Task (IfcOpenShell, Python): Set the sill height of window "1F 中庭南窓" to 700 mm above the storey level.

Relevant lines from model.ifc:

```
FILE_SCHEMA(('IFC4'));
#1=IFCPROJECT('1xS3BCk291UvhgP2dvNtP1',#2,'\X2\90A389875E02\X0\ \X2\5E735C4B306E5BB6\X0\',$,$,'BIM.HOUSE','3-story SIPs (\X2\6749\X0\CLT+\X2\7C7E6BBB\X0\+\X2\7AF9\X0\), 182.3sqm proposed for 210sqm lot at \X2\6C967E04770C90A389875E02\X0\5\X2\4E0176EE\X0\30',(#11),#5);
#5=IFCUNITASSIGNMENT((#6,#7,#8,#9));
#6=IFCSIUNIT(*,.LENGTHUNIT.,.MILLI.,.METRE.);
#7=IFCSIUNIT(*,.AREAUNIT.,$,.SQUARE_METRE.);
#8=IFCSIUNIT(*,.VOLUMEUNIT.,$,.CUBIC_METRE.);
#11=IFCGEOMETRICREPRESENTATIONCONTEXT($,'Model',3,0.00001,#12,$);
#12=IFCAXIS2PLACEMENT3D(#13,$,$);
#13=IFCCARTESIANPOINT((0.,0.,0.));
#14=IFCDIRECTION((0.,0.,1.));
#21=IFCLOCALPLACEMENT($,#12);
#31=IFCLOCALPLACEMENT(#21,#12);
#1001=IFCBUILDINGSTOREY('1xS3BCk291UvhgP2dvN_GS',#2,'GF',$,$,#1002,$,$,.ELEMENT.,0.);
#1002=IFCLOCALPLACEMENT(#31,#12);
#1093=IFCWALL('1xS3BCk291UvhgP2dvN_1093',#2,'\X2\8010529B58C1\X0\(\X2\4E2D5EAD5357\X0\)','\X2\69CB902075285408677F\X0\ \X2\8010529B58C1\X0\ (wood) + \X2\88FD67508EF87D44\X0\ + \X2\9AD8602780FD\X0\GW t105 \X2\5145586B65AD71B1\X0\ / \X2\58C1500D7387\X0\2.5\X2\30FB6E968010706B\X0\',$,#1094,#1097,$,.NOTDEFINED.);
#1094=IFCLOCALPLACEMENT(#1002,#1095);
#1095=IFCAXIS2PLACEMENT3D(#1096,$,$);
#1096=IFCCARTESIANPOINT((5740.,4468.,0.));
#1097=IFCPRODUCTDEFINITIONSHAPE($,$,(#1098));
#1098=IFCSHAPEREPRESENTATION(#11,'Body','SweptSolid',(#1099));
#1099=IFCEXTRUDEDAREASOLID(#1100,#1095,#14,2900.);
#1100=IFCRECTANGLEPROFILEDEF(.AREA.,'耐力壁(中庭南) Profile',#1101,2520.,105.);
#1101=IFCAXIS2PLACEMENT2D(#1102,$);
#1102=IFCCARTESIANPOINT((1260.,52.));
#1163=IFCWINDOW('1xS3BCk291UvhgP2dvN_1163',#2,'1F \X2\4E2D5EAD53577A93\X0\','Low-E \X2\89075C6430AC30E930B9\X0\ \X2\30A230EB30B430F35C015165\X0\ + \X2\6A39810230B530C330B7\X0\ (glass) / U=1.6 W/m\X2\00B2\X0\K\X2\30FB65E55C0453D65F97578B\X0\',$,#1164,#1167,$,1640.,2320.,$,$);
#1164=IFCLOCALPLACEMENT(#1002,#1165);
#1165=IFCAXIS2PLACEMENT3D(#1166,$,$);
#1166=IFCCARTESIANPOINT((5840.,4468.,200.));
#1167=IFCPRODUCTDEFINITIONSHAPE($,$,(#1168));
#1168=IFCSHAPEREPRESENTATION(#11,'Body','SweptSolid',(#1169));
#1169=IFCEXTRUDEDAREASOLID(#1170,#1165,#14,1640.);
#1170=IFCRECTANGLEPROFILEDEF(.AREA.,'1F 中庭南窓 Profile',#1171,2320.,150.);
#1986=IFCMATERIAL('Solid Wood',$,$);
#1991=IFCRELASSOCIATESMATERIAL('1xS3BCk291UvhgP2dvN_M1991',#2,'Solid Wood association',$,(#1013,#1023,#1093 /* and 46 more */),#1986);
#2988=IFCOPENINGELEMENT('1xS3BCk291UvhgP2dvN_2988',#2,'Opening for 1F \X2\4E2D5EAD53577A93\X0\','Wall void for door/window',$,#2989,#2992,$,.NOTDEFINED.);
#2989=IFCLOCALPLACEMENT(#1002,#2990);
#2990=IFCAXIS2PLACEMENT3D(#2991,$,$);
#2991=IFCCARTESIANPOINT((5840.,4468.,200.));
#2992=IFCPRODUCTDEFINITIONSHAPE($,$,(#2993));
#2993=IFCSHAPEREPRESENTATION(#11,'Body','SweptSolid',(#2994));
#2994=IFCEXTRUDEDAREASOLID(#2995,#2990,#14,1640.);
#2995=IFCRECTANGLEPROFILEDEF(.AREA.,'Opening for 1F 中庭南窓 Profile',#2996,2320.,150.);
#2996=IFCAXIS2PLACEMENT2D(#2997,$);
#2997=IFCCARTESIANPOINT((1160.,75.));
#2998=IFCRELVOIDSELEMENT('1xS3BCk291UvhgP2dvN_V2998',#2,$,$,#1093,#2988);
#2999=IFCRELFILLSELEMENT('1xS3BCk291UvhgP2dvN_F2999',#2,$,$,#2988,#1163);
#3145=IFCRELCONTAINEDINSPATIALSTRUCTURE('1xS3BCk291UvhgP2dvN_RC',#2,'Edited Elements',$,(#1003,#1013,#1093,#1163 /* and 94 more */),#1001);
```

```python
import numpy as np
import ifcopenshell
import ifcopenshell.api.geometry
import ifcopenshell.geom
import ifcopenshell.util.element
import ifcopenshell.util.placement
import ifcopenshell.util.shape
import ifcopenshell.util.unit

model = ifcopenshell.open("model.ifc")
unit_scale = ifcopenshell.util.unit.calculate_unit_scale(model)

window = model.by_guid("1xS3BCk291UvhgP2dvN_1163")
opening = window.FillsVoids[0].RelatingOpeningElement
storey = ifcopenshell.util.element.get_container(window, ifc_class="IfcBuildingStorey")
level = ifcopenshell.util.placement.get_local_placement(storey.ObjectPlacement)[2, 3]

# The opening's origin need not be at the sill, so measure its lowest point.
shape = ifcopenshell.geom.create_shape(ifcopenshell.geom.settings(), opening)
bottom = ifcopenshell.util.shape.get_shape_bottom_elevation(shape, shape.geometry) / unit_scale
dz = level + 0.7 / unit_scale - bottom

shift = np.array([0.0, 0.0, dz])
# The window is not placed relative to its opening, so move both.
for product in (opening, window):
    matrix = ifcopenshell.util.placement.get_local_placement(product.ObjectPlacement)
    matrix[:3, 3] += shift
    ifcopenshell.api.geometry.edit_object_placement(model, product=product, matrix=matrix, is_si=False)

print(f"moved by {dz * unit_scale:+.3f} m")

model.write("model_v2.ifc")
```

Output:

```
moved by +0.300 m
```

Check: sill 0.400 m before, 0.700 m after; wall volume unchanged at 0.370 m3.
